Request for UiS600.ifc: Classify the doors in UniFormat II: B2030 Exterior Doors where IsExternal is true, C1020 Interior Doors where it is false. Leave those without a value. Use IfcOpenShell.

First a look at what the model holds.

```python
import ifcopenshell
import ifcopenshell.util.element

model = ifcopenshell.open("UiS600.ifc")
print(model.schema)
print("classifications:", [c.Name for c in model.by_type("IfcClassification")])
values = [ifcopenshell.util.element.get_pset(e, "Pset_DoorCommon", "IsExternal") for e in model.by_type("IfcDoor")]
for value in (True, False, None):
    print("IsExternal", value, values.count(value))
```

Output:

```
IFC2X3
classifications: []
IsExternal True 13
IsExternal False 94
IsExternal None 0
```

```python
import ifcopenshell
import ifcopenshell.api.classification
import ifcopenshell.util.element

model = ifcopenshell.open("UiS600.ifc")

# IFC2X3 requires Source and Edition and has no link from the project to the system.
system = model.create_entity("IfcClassification", Source="ASTM", Edition="E1557", Name="UniFormat II")

doors = model.by_type("IfcDoor")
external = {e: ifcopenshell.util.element.get_pset(e, "Pset_DoorCommon", "IsExternal") for e in doors}
for flag, code, name in ((True, "B2030", "Exterior Doors"), (False, "C1020", "Interior Doors")):
    products = [e for e in doors if external[e] is flag]
    ifcopenshell.api.classification.add_reference(
        model, products=products, classification=system, identification=code, name=name
    )
    print(code, len(products))

model.write("UiS600_rev.ifc")
```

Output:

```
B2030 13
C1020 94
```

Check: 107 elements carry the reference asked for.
